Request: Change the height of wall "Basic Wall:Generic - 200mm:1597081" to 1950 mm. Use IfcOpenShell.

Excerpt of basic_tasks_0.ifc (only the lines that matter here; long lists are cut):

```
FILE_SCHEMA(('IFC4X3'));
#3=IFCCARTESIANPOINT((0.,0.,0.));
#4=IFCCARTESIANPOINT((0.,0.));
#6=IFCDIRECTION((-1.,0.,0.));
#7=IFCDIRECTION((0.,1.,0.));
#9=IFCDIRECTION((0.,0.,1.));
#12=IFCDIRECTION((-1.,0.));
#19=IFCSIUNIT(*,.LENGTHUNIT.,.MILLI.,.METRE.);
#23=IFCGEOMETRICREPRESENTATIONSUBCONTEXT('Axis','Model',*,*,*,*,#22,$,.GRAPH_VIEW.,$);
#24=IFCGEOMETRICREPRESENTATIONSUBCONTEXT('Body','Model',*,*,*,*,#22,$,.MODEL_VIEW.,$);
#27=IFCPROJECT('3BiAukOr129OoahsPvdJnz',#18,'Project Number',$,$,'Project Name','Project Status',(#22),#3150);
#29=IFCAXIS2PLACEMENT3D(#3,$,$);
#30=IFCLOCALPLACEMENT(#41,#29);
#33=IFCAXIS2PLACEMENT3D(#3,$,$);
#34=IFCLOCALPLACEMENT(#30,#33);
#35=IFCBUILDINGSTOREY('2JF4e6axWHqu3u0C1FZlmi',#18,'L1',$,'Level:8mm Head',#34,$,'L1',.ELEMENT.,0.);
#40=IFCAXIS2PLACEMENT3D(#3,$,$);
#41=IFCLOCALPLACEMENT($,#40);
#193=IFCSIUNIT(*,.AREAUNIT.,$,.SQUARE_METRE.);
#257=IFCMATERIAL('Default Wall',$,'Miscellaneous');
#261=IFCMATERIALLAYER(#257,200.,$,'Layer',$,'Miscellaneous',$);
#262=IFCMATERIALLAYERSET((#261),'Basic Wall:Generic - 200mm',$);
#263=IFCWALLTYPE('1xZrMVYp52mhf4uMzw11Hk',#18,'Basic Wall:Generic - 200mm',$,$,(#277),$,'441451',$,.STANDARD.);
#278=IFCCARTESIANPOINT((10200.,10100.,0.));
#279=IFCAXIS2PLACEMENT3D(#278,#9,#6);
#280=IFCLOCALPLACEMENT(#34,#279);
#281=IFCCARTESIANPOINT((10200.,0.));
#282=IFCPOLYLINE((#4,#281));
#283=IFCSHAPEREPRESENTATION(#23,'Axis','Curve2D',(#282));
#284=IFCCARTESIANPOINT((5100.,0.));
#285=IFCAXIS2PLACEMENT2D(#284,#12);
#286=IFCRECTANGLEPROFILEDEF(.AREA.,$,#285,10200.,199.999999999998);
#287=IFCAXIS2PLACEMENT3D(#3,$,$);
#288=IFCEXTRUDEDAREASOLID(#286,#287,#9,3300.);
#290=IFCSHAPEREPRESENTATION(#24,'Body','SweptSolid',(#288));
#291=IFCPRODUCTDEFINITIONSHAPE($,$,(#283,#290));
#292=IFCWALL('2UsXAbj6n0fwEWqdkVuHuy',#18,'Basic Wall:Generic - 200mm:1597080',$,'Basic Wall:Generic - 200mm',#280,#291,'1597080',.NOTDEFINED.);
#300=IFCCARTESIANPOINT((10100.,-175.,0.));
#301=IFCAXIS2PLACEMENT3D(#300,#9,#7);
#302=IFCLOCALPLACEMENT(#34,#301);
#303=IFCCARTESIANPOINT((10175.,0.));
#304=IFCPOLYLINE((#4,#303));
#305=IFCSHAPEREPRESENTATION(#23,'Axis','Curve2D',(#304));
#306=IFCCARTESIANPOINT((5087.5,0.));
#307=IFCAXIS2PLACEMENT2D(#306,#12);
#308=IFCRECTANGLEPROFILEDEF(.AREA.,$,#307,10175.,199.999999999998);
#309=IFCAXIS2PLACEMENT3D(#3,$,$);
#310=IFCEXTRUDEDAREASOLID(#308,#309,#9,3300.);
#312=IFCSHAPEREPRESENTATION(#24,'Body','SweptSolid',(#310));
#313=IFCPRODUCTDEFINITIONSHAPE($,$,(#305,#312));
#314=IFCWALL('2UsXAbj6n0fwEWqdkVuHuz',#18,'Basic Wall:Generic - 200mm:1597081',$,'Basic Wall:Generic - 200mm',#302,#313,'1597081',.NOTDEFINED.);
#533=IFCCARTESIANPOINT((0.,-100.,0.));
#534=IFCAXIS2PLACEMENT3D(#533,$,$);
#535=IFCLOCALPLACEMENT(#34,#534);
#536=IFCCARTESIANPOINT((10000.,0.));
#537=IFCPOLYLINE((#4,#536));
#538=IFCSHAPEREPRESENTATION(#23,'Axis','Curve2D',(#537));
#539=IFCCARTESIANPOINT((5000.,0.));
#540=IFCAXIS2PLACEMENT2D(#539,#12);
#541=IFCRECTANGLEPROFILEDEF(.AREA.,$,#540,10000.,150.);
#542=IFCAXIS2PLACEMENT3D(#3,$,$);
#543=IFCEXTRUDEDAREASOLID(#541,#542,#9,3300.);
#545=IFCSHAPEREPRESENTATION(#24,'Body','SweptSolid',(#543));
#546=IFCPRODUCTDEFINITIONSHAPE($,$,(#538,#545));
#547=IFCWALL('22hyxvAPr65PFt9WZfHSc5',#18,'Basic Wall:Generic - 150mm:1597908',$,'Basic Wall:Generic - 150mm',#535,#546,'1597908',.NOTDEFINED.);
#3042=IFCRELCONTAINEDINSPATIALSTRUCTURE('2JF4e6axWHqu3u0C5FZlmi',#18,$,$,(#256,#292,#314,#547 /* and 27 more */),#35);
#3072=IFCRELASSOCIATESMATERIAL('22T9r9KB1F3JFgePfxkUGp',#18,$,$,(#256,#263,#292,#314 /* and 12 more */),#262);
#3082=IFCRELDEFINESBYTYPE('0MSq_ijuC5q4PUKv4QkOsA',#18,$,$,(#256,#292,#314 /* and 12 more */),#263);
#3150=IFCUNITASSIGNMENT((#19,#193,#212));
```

```python
import ifcopenshell
import ifcopenshell.geom
import ifcopenshell.util.representation
import ifcopenshell.util.shape
import ifcopenshell.util.unit

model = ifcopenshell.open("basic_tasks_0.ifc")
unit_scale = ifcopenshell.util.unit.calculate_unit_scale(model)
settings = ifcopenshell.geom.settings()


def volume(element):
    """Net volume in cubic metres, openings subtracted."""
    shape = ifcopenshell.geom.create_shape(settings, element)
    return ifcopenshell.util.shape.get_volume(shape.geometry)


wall = model.by_id(314)
before = volume(wall)

body = ifcopenshell.util.representation.get_representation(wall, "Model", "Body")
solid = body.Items[0]
old_height = solid.Depth
solid.Depth = 1.95 / unit_scale
after = volume(wall)

print(f"height {old_height:g} -> {solid.Depth:g}, volume {before:.3f} -> {after:.3f} m3")

model.write("basic_tasks_0-out.ifc")
```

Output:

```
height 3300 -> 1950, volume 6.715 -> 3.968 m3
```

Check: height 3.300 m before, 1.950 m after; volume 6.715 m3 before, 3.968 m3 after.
